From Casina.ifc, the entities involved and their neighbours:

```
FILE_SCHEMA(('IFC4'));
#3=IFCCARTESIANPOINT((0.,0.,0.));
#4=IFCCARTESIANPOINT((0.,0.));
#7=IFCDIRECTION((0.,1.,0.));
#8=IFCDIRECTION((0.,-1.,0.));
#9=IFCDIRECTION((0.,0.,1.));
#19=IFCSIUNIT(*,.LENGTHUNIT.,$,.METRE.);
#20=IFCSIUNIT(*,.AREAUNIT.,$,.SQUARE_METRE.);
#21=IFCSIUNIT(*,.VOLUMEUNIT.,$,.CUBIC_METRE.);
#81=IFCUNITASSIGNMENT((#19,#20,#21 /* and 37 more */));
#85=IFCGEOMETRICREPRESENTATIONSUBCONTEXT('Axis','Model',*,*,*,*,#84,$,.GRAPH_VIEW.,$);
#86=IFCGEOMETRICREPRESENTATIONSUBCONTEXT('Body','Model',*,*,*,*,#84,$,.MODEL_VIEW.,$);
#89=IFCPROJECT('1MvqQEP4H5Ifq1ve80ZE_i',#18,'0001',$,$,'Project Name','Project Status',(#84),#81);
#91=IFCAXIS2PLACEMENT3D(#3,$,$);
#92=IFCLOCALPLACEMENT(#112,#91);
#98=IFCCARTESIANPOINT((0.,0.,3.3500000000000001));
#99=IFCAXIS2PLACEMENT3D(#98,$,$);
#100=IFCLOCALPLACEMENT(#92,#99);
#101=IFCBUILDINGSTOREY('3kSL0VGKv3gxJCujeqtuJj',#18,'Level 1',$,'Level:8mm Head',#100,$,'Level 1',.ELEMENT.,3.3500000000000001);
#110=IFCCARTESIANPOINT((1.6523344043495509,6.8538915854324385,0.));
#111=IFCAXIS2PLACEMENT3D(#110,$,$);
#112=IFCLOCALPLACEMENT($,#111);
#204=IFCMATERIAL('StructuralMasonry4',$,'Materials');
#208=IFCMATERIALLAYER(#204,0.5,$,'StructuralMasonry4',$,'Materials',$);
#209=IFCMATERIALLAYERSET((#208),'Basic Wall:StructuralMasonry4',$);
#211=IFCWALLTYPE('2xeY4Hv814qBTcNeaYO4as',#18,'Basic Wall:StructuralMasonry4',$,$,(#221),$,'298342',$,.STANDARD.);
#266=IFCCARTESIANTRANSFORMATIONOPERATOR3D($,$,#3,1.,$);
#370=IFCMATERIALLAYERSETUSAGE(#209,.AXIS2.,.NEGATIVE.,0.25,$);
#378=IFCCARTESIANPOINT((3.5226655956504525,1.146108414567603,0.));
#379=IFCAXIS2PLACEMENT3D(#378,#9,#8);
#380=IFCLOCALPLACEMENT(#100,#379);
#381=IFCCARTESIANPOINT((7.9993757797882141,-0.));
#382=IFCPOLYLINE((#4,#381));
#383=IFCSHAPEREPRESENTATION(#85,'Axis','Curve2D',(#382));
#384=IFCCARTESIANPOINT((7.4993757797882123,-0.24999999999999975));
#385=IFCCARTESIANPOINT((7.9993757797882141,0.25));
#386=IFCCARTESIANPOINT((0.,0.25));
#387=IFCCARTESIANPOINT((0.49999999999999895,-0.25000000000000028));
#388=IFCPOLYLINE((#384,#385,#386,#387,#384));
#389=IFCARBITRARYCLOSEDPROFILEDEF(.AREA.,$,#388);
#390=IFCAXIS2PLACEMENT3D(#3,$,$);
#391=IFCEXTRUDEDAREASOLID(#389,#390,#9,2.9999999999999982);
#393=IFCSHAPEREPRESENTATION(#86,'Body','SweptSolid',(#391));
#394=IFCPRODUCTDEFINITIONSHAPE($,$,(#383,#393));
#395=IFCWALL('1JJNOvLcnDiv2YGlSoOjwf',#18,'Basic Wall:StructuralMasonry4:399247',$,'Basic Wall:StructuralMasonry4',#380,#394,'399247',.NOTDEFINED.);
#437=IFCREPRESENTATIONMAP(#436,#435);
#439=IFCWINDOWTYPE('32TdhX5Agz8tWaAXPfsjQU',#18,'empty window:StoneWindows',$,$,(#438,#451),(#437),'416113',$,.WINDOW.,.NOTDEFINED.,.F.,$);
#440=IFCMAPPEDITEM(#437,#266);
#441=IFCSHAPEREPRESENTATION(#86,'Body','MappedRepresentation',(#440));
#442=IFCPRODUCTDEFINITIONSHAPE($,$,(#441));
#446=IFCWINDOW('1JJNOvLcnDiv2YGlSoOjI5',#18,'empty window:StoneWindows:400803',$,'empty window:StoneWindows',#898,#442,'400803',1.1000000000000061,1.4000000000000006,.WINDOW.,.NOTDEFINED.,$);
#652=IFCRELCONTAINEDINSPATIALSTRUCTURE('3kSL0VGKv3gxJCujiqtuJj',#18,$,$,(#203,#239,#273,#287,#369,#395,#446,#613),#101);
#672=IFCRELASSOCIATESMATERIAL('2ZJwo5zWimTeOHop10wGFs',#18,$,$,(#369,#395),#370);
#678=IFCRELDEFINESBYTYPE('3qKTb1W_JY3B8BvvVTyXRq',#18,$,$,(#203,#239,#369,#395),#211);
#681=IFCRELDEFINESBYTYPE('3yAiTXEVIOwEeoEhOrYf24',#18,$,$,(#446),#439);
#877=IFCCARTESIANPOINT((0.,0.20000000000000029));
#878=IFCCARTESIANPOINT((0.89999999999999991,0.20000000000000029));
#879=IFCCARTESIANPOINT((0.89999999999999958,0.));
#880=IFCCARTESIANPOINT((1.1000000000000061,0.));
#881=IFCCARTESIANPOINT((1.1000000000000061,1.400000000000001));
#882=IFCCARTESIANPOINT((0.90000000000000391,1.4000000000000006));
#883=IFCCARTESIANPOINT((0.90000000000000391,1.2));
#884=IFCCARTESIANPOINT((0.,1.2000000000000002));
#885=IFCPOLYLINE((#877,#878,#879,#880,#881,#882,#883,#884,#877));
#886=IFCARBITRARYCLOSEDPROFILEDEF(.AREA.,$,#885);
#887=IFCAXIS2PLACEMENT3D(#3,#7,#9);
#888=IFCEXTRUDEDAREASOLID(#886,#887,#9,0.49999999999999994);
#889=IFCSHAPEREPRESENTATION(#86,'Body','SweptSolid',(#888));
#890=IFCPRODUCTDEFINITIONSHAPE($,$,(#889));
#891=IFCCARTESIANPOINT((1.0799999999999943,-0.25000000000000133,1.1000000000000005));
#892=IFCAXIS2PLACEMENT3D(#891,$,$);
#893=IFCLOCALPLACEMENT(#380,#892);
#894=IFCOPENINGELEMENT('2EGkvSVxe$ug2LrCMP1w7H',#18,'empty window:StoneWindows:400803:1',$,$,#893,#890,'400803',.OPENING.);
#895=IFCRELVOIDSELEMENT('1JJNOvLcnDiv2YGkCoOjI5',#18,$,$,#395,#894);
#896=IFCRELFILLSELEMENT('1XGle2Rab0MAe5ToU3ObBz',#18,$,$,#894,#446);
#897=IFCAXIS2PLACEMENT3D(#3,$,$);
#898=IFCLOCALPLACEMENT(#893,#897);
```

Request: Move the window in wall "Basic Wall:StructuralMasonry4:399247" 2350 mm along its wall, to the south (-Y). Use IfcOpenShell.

```python
import ifcopenshell
import ifcopenshell.api.geometry
import ifcopenshell.util.placement

model = ifcopenshell.open("Casina.ifc")

window = model.by_guid("1JJNOvLcnDiv2YGlSoOjI5")
opening = window.FillsVoids[0].RelatingOpeningElement
wall = opening.VoidsElements[0].RelatingBuildingElement

wall_matrix = ifcopenshell.util.placement.get_local_placement(wall.ObjectPlacement)
shift = wall_matrix[:3, 0] * 2.35
before = ifcopenshell.util.placement.get_local_placement(window.ObjectPlacement)[:3, 3].copy()

# The window is placed relative to its opening, so it follows when the opening moves.
matrix = ifcopenshell.util.placement.get_local_placement(opening.ObjectPlacement)
matrix[:3, 3] += shift
ifcopenshell.api.geometry.edit_object_placement(
    model, product=opening, matrix=matrix, is_si=False, should_transform_children=True
)

after = ifcopenshell.util.placement.get_local_placement(window.ObjectPlacement)[:3, 3]
print("window moved by", (after - before).round(3) + 0.0)

model.write("Casina_v2.ifc")
```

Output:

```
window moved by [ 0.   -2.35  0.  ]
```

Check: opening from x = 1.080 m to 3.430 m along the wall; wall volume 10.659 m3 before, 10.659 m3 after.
